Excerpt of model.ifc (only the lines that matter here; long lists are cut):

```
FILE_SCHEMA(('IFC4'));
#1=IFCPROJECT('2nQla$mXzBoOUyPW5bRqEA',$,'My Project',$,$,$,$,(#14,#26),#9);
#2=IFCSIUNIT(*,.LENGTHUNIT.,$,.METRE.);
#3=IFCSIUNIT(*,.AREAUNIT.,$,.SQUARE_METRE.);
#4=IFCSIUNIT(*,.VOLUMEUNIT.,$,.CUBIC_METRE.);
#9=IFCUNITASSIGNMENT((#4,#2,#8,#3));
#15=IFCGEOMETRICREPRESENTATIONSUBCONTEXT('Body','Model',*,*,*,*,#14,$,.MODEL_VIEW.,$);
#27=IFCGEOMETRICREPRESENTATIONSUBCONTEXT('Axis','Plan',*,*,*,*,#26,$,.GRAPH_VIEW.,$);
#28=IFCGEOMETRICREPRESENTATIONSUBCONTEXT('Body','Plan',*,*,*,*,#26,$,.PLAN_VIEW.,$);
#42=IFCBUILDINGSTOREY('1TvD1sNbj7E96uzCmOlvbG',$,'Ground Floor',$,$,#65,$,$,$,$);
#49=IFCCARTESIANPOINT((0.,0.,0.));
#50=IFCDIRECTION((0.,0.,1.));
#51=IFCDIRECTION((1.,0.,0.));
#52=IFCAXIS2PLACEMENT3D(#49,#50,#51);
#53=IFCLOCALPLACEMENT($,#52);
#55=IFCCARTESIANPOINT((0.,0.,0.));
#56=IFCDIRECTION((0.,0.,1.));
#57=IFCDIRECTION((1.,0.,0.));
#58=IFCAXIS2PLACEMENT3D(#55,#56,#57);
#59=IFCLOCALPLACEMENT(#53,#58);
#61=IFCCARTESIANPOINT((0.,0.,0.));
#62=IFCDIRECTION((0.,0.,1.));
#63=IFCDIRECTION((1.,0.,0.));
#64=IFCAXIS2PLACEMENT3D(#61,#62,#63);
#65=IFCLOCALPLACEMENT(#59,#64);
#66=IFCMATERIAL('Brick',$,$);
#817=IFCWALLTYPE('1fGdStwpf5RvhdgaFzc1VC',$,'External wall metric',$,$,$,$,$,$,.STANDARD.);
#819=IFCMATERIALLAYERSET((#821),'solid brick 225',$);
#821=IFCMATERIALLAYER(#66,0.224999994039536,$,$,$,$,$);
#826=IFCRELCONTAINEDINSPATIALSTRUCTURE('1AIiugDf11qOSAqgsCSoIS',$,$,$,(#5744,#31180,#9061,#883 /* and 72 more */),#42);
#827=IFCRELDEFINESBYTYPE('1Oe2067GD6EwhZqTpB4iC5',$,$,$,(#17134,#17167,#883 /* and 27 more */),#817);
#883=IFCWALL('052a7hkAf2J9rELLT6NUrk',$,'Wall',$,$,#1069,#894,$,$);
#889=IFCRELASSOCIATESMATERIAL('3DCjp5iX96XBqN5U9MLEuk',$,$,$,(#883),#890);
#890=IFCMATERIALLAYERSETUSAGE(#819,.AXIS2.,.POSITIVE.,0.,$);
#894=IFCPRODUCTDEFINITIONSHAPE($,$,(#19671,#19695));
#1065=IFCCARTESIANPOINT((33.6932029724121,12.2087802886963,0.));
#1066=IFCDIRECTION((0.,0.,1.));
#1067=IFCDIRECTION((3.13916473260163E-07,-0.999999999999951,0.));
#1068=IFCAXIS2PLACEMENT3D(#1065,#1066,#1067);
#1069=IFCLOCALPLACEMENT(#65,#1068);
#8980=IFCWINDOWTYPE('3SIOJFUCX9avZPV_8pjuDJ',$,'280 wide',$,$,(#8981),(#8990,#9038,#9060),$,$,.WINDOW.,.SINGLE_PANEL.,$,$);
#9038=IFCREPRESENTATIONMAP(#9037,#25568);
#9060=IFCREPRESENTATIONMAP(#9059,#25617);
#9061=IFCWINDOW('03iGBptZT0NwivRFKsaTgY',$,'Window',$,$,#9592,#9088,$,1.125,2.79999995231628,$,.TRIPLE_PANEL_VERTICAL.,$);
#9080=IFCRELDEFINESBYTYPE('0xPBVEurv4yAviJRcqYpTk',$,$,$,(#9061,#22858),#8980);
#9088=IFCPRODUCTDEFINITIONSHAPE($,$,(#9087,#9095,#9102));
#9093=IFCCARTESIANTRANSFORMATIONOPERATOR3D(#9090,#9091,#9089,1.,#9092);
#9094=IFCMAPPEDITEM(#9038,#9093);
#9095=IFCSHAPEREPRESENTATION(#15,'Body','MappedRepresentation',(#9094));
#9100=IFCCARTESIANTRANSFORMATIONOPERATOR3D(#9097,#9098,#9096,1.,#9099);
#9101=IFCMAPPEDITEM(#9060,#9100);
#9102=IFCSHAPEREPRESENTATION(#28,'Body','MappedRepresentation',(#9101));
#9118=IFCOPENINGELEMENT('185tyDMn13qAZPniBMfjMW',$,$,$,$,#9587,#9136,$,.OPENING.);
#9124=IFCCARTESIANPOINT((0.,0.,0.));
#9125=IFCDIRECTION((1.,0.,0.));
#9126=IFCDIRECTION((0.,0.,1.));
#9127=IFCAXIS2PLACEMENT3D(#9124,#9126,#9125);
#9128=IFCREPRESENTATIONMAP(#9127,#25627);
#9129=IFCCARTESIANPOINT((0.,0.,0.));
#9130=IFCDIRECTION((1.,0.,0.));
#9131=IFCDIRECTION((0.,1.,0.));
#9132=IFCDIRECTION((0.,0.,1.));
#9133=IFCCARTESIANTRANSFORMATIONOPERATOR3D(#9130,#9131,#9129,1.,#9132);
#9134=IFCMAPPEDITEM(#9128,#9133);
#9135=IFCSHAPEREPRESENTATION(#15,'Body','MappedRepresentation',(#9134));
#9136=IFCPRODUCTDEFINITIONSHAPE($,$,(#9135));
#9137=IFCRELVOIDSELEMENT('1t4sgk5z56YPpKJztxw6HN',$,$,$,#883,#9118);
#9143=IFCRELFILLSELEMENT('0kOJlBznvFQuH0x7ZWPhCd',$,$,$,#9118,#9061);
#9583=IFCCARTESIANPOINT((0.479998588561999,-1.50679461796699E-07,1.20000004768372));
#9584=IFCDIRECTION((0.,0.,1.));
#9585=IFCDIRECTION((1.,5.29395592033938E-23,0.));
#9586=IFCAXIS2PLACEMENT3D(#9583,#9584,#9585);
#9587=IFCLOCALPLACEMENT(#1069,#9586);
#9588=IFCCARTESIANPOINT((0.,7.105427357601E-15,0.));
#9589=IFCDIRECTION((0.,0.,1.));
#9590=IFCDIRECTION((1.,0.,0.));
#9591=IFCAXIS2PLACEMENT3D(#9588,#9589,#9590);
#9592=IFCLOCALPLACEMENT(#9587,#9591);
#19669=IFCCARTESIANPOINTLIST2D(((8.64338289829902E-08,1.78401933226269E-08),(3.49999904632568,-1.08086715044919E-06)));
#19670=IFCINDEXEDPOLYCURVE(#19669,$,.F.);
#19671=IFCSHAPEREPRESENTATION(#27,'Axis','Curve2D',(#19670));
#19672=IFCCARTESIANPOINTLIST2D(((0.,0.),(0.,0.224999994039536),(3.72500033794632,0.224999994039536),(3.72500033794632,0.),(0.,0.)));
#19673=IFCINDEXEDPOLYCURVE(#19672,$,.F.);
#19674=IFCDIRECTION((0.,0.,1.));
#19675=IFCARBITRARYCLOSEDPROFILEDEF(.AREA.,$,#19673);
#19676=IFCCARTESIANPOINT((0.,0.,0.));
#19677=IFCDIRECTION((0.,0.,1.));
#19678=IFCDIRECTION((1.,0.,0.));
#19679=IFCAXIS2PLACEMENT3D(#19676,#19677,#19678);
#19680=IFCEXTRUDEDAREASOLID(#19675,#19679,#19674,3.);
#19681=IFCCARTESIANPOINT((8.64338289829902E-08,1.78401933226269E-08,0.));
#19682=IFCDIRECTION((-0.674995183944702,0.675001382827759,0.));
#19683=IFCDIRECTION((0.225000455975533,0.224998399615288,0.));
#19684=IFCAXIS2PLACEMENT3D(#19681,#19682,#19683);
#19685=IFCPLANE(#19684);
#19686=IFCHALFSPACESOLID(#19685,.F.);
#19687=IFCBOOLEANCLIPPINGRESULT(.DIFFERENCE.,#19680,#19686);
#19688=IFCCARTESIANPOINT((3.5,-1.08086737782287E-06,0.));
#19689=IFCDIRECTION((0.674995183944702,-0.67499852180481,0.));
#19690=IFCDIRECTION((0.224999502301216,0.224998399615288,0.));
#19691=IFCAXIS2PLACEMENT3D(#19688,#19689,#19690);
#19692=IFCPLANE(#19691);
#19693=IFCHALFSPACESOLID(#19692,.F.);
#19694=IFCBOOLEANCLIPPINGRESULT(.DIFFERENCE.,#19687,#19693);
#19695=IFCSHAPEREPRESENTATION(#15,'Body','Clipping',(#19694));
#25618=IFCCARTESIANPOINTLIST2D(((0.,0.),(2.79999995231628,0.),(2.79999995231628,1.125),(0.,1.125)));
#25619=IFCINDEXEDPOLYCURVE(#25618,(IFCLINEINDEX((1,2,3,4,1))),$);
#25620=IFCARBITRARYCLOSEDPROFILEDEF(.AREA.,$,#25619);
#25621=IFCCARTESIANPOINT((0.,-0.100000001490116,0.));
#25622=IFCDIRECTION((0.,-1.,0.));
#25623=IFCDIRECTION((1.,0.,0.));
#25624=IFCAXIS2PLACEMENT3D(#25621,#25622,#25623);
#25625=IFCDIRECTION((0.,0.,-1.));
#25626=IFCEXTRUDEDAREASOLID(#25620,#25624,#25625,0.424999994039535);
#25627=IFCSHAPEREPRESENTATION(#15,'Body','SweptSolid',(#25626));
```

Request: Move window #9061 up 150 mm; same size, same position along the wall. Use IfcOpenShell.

```python
import numpy as np
import ifcopenshell
import ifcopenshell.api.geometry
import ifcopenshell.util.placement
import ifcopenshell.util.unit

model = ifcopenshell.open("model.ifc")
unit_scale = ifcopenshell.util.unit.calculate_unit_scale(model)

window = model.by_guid("03iGBptZT0NwivRFKsaTgY")
opening = window.FillsVoids[0].RelatingOpeningElement
dz = 0.15

shift = np.array([0.0, 0.0, dz])
# The window is placed relative to its opening, so it follows when the opening moves.
matrix = ifcopenshell.util.placement.get_local_placement(opening.ObjectPlacement)
matrix[:3, 3] += shift
ifcopenshell.api.geometry.edit_object_placement(
    model, product=opening, matrix=matrix, is_si=False, should_transform_children=True
)

print(f"moved by {dz * unit_scale:+.3f} m")

model.write("model_rev.ifc")
```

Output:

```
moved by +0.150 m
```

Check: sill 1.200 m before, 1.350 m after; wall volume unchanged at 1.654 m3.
